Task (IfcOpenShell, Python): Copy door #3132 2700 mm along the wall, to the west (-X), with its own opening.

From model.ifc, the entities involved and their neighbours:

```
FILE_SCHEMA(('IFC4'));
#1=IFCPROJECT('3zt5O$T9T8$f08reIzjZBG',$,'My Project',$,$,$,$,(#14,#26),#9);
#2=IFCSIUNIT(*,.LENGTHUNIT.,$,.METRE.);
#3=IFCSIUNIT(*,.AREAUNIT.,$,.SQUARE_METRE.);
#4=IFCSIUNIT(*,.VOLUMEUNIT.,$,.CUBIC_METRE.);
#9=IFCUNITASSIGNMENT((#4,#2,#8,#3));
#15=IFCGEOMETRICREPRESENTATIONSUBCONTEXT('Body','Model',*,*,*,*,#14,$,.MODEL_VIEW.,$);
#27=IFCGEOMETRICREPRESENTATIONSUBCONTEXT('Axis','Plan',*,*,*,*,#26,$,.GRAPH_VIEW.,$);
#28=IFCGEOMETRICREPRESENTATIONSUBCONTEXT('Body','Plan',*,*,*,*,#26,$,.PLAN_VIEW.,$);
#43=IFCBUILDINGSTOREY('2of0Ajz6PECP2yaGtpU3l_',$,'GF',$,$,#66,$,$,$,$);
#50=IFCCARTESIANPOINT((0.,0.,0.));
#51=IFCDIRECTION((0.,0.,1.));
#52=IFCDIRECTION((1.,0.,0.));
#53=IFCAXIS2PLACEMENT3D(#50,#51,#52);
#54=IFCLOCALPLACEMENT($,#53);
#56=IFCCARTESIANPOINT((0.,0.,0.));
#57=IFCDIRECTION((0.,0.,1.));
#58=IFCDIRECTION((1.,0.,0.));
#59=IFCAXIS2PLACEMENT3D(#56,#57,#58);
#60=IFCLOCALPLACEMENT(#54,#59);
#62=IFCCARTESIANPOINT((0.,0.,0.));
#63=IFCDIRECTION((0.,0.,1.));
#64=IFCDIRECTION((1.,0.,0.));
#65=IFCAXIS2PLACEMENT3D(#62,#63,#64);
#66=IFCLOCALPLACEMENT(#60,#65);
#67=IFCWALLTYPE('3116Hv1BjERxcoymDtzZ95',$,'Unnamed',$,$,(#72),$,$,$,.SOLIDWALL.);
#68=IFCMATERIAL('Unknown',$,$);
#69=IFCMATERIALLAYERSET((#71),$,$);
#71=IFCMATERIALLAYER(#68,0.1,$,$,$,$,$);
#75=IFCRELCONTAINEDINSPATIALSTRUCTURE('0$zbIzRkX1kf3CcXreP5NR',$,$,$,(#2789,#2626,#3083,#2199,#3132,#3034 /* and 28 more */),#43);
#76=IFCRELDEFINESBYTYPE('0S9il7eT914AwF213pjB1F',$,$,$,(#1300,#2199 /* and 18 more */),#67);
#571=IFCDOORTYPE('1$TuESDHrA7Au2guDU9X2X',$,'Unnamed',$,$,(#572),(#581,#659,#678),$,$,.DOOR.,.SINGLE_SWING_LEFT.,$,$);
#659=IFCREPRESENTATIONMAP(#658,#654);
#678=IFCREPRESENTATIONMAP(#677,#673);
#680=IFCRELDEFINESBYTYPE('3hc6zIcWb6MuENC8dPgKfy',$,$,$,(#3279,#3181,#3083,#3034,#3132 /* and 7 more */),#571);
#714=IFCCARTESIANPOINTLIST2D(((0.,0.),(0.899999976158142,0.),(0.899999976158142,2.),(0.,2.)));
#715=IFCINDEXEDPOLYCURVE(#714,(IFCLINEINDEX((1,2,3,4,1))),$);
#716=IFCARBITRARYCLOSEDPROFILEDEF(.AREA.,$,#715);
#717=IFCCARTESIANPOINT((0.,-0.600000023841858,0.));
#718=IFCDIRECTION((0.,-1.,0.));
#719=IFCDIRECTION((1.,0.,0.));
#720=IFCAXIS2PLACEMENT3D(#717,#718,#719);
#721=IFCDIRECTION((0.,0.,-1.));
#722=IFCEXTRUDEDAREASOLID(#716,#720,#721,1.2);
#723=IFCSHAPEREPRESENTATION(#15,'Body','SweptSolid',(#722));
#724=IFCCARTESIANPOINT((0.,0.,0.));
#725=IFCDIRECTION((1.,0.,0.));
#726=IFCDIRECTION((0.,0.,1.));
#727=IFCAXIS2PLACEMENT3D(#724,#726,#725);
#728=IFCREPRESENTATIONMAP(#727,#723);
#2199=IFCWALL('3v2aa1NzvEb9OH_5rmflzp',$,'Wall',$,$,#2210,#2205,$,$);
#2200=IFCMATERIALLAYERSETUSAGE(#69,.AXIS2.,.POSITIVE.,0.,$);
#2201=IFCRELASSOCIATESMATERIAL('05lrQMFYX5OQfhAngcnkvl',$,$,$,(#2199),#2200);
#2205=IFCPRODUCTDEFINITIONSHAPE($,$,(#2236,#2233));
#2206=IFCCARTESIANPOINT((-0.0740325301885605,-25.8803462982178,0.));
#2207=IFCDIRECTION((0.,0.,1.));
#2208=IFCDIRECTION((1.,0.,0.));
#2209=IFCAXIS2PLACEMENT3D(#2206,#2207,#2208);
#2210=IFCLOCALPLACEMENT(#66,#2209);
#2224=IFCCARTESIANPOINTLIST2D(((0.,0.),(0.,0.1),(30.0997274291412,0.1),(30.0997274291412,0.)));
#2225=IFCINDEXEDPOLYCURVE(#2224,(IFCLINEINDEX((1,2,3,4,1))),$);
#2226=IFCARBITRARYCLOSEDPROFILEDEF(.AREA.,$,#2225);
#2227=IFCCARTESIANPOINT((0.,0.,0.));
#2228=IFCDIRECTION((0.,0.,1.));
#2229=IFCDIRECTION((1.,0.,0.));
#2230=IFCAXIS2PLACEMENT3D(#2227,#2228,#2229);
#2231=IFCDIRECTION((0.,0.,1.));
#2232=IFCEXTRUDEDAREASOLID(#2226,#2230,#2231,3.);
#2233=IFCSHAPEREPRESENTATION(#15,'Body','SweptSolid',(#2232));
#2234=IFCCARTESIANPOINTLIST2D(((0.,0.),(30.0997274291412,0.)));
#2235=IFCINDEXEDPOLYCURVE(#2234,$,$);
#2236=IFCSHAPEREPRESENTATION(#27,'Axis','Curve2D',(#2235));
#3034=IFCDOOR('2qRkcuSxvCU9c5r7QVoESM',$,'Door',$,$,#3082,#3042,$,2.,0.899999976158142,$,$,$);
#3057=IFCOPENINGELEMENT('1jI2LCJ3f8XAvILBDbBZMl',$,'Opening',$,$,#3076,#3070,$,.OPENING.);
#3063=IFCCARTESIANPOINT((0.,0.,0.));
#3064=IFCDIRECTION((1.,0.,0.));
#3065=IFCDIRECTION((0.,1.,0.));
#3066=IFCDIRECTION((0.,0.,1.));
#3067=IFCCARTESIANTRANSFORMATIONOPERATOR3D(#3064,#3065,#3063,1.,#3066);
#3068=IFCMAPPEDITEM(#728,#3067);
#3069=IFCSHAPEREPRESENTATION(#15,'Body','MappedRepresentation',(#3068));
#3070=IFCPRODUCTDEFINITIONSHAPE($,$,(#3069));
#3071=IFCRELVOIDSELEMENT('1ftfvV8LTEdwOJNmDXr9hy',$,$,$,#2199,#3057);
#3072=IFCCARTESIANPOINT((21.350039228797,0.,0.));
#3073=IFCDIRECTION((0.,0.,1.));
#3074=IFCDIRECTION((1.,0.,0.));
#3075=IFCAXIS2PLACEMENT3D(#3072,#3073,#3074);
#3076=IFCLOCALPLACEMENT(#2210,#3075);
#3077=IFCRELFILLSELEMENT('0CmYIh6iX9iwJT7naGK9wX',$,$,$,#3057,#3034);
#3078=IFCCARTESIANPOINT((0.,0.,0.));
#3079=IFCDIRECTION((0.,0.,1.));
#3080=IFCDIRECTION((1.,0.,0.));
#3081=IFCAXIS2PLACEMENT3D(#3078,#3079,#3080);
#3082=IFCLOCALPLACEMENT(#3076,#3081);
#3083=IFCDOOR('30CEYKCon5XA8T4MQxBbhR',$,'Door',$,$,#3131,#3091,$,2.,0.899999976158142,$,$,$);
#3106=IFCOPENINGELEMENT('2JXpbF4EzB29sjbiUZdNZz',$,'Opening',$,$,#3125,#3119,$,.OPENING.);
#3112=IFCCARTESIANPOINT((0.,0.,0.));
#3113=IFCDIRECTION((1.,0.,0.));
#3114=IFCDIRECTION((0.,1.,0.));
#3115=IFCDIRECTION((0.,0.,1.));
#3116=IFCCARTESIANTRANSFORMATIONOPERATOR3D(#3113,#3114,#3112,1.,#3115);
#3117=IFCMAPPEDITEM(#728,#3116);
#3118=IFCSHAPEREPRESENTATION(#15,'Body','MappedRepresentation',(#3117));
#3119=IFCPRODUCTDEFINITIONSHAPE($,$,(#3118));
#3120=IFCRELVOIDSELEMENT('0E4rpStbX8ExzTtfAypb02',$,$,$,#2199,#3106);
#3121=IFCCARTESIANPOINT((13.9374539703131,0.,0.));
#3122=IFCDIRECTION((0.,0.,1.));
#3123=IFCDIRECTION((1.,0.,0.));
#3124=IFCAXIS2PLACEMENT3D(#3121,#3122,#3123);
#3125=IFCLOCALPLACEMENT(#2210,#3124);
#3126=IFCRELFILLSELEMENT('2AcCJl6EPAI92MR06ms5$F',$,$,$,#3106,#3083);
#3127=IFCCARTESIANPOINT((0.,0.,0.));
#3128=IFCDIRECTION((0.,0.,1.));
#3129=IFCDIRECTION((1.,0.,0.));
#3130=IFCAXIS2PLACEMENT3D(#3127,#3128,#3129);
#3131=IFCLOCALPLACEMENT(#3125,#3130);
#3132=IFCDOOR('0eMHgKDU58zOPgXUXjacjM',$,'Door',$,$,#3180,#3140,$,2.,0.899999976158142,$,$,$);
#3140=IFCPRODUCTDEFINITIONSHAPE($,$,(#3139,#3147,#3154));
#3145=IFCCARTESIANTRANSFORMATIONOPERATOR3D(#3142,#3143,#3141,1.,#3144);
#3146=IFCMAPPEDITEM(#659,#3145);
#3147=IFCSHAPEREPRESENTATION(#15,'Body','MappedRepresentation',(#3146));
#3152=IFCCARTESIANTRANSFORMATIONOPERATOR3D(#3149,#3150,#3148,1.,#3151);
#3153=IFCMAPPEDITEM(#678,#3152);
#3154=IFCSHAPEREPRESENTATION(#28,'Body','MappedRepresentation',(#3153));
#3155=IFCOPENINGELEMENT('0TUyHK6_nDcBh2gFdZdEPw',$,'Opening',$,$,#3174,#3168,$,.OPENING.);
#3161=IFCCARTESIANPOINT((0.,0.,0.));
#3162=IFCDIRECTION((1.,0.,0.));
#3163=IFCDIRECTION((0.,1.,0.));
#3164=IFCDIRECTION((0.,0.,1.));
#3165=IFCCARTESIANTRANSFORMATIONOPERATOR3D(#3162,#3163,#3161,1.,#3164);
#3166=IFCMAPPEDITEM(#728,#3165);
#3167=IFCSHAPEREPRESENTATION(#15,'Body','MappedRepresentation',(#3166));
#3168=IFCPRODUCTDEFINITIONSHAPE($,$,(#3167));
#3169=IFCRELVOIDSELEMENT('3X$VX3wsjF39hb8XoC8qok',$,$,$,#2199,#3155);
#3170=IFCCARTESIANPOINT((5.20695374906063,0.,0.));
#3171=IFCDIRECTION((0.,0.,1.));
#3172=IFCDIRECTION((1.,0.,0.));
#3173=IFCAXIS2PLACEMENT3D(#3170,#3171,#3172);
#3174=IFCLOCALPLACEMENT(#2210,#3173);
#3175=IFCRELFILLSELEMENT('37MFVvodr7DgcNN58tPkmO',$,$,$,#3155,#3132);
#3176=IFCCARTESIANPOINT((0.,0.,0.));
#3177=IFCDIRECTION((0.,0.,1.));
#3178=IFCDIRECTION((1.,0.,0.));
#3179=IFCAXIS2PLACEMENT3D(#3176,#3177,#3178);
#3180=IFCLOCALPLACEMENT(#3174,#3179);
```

```python
import ifcopenshell
import ifcopenshell.api.feature
import ifcopenshell.api.geometry
import ifcopenshell.api.root
import ifcopenshell.geom
import ifcopenshell.util.element
import ifcopenshell.util.placement
import ifcopenshell.util.shape

model = ifcopenshell.open("model.ifc")
settings = ifcopenshell.geom.settings()


def volume(element):
    """Net volume in cubic metres, openings subtracted."""
    shape = ifcopenshell.geom.create_shape(settings, element)
    return ifcopenshell.util.shape.get_volume(shape.geometry)


door = model.by_guid("0eMHgKDU58zOPgXUXjacjM")
opening = door.FillsVoids[0].RelatingOpeningElement
wall = opening.VoidsElements[0].RelatingBuildingElement
before = volume(wall)
shift = ifcopenshell.util.placement.get_local_placement(wall.ObjectPlacement)[:3, 0] * -2.7

# copy_class copies the void relationship, type, container and properties, but no geometry.
new_opening = ifcopenshell.api.root.copy_class(model, product=opening)
new_opening.Representation = ifcopenshell.util.element.copy_deep(
    model, opening.Representation, exclude=["IfcGeometricRepresentationContext", "IfcRepresentationMap"]
)
new_door = ifcopenshell.api.root.copy_class(model, product=door)
new_door.Representation = ifcopenshell.util.element.copy_deep(
    model, door.Representation, exclude=["IfcGeometricRepresentationContext", "IfcRepresentationMap"]
)
ifcopenshell.api.feature.add_filling(model, opening=new_opening, element=new_door)

for old, new in ((opening, new_opening), (door, new_door)):
    matrix = ifcopenshell.util.placement.get_local_placement(old.ObjectPlacement)
    matrix[:3, 3] += shift
    ifcopenshell.api.geometry.edit_object_placement(model, product=new, matrix=matrix, is_si=False)

after = volume(wall)

print(f"wall volume {before:.3f} -> {after:.3f} m3")

model.write("model_updated.ifc")
```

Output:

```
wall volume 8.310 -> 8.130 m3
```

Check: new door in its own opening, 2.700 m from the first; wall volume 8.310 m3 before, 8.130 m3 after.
